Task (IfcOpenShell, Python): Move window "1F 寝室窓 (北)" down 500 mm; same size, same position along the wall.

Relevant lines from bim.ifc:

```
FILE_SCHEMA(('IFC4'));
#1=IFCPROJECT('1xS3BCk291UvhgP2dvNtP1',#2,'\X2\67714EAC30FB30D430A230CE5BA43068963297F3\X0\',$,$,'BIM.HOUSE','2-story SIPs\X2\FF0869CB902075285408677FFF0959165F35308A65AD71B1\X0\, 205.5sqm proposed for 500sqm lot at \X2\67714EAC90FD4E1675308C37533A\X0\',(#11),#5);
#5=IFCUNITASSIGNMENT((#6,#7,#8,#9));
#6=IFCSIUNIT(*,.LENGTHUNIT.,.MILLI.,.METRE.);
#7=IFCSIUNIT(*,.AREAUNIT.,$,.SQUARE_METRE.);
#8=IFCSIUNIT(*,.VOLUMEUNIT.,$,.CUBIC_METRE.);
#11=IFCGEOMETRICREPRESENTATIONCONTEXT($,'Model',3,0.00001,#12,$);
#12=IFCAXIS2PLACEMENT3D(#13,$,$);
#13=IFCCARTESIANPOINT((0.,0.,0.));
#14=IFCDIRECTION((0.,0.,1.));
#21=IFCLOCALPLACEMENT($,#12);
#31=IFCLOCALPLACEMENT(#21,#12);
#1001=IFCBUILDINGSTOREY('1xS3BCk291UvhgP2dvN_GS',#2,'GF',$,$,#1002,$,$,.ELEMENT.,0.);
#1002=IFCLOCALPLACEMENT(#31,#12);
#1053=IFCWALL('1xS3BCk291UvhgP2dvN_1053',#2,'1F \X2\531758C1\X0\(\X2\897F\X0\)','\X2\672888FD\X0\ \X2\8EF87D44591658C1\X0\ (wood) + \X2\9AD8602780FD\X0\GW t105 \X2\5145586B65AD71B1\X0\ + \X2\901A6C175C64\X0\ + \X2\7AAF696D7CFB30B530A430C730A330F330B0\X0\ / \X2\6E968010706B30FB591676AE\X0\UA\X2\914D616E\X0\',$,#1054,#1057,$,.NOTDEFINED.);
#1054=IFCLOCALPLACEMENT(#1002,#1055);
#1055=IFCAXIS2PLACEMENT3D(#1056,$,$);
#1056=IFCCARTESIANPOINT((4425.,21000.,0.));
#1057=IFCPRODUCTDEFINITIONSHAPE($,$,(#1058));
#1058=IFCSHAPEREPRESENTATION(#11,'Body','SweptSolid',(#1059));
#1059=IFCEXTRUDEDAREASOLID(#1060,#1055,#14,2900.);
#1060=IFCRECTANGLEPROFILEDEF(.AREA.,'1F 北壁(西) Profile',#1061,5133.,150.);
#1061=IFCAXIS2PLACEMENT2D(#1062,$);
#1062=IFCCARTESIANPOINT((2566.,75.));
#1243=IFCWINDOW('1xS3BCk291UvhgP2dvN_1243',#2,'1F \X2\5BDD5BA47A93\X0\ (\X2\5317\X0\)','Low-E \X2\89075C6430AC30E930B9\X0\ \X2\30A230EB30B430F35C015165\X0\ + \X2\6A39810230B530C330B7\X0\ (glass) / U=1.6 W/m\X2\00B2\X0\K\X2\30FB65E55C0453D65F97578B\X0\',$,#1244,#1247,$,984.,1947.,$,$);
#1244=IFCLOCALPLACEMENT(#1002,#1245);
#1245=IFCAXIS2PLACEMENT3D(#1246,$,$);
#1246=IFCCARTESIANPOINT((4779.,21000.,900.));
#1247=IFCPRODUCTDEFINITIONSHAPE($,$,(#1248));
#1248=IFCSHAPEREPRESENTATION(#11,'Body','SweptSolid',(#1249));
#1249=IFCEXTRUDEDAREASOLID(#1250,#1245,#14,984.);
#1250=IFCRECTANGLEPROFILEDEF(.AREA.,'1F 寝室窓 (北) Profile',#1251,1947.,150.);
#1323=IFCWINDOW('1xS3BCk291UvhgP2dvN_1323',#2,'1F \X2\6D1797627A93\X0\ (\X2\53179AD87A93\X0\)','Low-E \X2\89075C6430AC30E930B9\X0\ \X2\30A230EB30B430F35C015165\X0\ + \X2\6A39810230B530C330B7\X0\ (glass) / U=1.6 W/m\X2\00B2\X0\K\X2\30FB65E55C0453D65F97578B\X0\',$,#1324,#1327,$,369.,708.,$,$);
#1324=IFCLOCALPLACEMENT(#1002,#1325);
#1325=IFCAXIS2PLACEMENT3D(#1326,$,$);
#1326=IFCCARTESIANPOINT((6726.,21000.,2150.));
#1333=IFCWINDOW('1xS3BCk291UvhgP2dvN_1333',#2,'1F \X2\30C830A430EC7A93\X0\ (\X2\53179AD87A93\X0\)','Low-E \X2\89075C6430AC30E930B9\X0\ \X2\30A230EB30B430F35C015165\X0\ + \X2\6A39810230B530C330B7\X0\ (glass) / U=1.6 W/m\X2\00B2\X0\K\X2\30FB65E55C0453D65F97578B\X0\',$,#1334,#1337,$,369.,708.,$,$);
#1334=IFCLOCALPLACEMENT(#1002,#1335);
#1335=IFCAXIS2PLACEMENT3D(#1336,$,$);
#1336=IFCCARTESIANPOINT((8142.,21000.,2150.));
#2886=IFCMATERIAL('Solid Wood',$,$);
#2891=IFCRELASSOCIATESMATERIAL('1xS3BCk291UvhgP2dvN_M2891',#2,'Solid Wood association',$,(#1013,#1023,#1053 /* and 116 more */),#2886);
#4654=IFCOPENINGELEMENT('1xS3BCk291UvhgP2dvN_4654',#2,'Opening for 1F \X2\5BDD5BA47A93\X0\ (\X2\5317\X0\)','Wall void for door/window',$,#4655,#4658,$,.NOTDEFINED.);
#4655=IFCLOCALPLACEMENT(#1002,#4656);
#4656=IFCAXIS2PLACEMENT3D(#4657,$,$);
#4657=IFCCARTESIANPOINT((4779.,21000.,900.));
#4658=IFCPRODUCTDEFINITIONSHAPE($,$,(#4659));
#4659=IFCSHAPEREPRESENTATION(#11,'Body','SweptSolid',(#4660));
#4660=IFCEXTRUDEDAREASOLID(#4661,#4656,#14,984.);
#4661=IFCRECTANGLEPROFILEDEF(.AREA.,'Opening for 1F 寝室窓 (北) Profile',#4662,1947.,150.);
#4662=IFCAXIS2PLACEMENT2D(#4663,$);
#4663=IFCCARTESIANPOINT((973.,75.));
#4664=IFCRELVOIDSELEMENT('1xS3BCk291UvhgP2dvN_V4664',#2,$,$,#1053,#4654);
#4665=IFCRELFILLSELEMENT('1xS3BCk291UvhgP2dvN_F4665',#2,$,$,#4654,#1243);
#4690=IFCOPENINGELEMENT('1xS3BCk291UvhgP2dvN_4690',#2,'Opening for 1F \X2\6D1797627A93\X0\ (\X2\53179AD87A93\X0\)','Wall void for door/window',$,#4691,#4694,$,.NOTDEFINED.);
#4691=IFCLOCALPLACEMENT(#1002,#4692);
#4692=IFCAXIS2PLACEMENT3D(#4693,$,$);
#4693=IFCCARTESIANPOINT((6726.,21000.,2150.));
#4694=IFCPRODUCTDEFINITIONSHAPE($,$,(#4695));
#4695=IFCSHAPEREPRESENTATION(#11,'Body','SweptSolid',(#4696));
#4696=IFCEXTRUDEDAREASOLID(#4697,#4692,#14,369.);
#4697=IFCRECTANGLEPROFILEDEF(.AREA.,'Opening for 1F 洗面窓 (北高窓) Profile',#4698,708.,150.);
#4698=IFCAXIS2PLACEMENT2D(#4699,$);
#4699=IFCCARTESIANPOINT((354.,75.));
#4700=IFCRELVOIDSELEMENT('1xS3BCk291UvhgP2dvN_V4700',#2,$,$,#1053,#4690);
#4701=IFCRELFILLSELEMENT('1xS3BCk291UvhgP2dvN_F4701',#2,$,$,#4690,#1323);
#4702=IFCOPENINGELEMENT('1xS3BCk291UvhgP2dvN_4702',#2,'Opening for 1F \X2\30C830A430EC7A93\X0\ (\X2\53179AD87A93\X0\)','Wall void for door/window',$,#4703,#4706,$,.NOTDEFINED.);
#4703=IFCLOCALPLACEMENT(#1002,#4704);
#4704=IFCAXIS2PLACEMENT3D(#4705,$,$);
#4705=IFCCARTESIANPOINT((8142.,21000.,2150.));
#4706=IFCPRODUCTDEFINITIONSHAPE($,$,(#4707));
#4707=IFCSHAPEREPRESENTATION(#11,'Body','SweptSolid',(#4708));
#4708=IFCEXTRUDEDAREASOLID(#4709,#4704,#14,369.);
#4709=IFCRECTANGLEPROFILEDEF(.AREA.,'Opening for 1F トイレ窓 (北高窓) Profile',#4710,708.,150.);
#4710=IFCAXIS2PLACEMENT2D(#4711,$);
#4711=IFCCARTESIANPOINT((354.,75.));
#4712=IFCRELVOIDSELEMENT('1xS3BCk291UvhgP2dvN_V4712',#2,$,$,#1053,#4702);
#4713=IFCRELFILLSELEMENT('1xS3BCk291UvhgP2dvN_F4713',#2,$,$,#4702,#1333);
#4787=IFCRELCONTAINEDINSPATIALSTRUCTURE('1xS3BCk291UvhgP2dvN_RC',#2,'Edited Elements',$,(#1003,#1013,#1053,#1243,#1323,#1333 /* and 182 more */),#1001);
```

```python
import numpy as np
import ifcopenshell
import ifcopenshell.api.geometry
import ifcopenshell.util.placement
import ifcopenshell.util.unit

model = ifcopenshell.open("bim.ifc")
unit_scale = ifcopenshell.util.unit.calculate_unit_scale(model)

window = model.by_id(1243)
opening = window.FillsVoids[0].RelatingOpeningElement
dz = -0.5 / unit_scale

shift = np.array([0.0, 0.0, dz])
# The window is not placed relative to its opening, so move both.
for product in (opening, window):
    matrix = ifcopenshell.util.placement.get_local_placement(product.ObjectPlacement)
    matrix[:3, 3] += shift
    ifcopenshell.api.geometry.edit_object_placement(model, product=product, matrix=matrix, is_si=False)

print(f"moved by {dz * unit_scale:+.3f} m")

model.write("bim_edited.ifc")
```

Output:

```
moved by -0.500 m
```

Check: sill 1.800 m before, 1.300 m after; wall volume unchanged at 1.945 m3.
